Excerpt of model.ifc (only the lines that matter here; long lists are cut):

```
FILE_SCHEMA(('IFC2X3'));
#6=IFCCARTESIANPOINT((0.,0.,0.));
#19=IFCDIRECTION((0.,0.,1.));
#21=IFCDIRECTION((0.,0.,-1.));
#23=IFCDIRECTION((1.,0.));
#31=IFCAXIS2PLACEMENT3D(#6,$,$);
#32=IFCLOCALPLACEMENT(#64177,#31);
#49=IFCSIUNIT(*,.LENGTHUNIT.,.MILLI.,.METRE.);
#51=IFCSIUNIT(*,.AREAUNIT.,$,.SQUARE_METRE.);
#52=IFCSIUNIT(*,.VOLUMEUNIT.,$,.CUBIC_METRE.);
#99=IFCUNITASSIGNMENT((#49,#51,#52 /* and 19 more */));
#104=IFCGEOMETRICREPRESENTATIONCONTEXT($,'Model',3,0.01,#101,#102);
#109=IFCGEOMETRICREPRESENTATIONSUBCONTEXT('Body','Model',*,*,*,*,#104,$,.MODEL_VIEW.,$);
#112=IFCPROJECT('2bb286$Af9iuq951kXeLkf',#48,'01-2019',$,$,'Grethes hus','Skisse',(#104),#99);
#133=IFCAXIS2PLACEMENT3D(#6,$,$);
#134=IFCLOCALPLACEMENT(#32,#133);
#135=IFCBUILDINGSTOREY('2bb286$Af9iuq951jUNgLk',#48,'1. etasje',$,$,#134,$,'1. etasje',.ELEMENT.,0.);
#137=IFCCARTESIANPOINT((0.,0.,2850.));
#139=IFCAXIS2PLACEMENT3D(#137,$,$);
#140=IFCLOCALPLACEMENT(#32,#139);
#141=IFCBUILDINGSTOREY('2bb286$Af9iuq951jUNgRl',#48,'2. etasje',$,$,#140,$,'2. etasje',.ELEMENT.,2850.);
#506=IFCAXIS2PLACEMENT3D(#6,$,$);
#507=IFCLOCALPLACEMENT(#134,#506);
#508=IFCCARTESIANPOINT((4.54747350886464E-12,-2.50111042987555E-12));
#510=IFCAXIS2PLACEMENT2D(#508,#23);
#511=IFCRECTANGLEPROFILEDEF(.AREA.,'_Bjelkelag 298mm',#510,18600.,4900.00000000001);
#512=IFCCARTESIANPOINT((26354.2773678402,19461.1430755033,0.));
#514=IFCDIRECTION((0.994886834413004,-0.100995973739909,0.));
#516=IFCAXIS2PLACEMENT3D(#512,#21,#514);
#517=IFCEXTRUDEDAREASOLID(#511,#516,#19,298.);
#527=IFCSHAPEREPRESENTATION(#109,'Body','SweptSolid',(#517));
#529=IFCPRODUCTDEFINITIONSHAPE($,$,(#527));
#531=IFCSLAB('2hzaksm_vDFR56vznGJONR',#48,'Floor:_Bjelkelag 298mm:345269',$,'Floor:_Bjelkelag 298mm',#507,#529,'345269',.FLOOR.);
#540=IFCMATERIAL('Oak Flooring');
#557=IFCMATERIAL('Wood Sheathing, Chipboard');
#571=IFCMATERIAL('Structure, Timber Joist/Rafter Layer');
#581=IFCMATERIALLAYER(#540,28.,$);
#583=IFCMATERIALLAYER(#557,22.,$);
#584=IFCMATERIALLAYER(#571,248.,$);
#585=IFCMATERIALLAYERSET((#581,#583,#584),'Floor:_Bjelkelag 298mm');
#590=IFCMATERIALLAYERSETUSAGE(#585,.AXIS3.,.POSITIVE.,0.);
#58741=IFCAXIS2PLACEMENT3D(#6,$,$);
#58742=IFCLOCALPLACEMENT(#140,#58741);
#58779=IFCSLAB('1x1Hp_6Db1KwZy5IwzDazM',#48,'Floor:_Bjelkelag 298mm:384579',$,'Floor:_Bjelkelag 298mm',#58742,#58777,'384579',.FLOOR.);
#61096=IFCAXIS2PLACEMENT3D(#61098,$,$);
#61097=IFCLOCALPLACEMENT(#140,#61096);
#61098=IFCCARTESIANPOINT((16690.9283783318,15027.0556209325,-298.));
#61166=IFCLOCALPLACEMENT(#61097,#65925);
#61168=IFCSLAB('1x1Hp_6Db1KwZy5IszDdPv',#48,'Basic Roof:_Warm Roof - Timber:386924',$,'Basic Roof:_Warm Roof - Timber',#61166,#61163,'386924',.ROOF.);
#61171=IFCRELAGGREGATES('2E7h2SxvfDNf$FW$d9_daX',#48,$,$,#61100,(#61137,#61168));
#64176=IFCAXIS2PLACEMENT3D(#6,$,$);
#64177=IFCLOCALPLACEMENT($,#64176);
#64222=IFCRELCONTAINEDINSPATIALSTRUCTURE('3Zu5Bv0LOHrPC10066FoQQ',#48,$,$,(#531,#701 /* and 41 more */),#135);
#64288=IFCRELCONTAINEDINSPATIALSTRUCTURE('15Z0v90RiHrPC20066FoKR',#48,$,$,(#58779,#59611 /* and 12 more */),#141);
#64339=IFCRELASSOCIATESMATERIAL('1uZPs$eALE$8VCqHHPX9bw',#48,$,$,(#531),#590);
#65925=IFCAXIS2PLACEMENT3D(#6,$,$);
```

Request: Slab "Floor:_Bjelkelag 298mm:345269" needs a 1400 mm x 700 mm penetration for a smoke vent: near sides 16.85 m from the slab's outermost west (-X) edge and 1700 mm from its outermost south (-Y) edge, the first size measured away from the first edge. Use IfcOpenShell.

```python
import numpy as np
import ifcopenshell
import ifcopenshell.api.feature
import ifcopenshell.api.geometry
import ifcopenshell.api.root
import ifcopenshell.geom
import ifcopenshell.util.placement
import ifcopenshell.util.representation
import ifcopenshell.util.shape
import ifcopenshell.util.unit

model = ifcopenshell.open("model.ifc")
unit_scale = ifcopenshell.util.unit.calculate_unit_scale(model)
settings = ifcopenshell.geom.settings()


def volume(element):
    """Net volume in cubic metres, openings subtracted."""
    shape = ifcopenshell.geom.create_shape(settings, element)
    return ifcopenshell.util.shape.get_volume(shape.geometry)


slab = model.by_guid("2hzaksm_vDFR56vznGJONR")
before = volume(slab)

# Extent in the slab's own axes, in metres. The edges named are its -X and -Y sides.
slab_shape = ifcopenshell.geom.create_shape(settings, slab)
vertices = ifcopenshell.util.shape.get_vertices(slab_shape.geometry)
x_min, y_min, bottom = vertices.min(axis=0)
top = vertices[:, 2].max()

opening = ifcopenshell.api.root.create_entity(model, ifc_class="IfcOpeningElement", name="Smoke vent opening")
context = ifcopenshell.util.representation.get_context(model, "Model", "Body", "MODEL_VIEW")
width, depth = 1.4, 0.7
outline = [(0.0, 0.0), (width, 0.0), (width, depth), (0.0, depth), (0.0, 0.0)]
# Overshoot both faces by 50 mm so the cut is clean.
shape = ifcopenshell.api.geometry.add_slab_representation(
    model, context=context, depth=top - bottom + 0.1, polyline=outline
)
ifcopenshell.api.geometry.assign_representation(model, product=opening, representation=shape)

matrix = ifcopenshell.util.placement.get_local_placement(slab.ObjectPlacement)
matrix[:, 3] = matrix @ np.append(np.array([x_min + 16.85, y_min + 1.7, bottom - 0.05]) / unit_scale, 1.0)
ifcopenshell.api.geometry.edit_object_placement(model, product=opening, matrix=matrix, is_si=False)
ifcopenshell.api.feature.add_feature(model, feature=opening, element=slab)

after = volume(slab)

print(f"slab volume {before:.3f} -> {after:.3f} m3")

model.write("model_edited.ifc")
```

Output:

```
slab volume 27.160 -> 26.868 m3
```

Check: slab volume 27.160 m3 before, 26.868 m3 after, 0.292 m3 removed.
